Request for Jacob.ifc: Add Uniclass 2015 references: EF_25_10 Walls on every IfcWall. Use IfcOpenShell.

First a look at what the model holds.

```python
import ifcopenshell

model = ifcopenshell.open("Jacob.ifc")
print(model.schema)
print("classifications:", [c.Name for c in model.by_type("IfcClassification")])
for ifc_class in ("IfcDoor", "IfcRoof", "IfcStair", "IfcWall", "IfcWindow"):
    print(ifc_class, len(model.by_type(ifc_class)))
```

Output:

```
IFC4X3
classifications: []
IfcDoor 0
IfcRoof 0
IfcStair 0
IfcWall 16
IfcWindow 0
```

```python
import ifcopenshell
import ifcopenshell.api.classification

model = ifcopenshell.open("Jacob.ifc")

system = ifcopenshell.api.classification.add_classification(model, classification="Uniclass 2015")

codes = {
    "IfcWall": ("EF_25_10", "Walls"),
}
for ifc_class, (code, name) in codes.items():
    products = model.by_type(ifc_class)
    ifcopenshell.api.classification.add_reference(
        model, products=products, classification=system, identification=code, name=name
    )
    print(code, len(products))

model.write("Jacob-out.ifc")
```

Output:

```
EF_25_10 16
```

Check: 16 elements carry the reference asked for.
